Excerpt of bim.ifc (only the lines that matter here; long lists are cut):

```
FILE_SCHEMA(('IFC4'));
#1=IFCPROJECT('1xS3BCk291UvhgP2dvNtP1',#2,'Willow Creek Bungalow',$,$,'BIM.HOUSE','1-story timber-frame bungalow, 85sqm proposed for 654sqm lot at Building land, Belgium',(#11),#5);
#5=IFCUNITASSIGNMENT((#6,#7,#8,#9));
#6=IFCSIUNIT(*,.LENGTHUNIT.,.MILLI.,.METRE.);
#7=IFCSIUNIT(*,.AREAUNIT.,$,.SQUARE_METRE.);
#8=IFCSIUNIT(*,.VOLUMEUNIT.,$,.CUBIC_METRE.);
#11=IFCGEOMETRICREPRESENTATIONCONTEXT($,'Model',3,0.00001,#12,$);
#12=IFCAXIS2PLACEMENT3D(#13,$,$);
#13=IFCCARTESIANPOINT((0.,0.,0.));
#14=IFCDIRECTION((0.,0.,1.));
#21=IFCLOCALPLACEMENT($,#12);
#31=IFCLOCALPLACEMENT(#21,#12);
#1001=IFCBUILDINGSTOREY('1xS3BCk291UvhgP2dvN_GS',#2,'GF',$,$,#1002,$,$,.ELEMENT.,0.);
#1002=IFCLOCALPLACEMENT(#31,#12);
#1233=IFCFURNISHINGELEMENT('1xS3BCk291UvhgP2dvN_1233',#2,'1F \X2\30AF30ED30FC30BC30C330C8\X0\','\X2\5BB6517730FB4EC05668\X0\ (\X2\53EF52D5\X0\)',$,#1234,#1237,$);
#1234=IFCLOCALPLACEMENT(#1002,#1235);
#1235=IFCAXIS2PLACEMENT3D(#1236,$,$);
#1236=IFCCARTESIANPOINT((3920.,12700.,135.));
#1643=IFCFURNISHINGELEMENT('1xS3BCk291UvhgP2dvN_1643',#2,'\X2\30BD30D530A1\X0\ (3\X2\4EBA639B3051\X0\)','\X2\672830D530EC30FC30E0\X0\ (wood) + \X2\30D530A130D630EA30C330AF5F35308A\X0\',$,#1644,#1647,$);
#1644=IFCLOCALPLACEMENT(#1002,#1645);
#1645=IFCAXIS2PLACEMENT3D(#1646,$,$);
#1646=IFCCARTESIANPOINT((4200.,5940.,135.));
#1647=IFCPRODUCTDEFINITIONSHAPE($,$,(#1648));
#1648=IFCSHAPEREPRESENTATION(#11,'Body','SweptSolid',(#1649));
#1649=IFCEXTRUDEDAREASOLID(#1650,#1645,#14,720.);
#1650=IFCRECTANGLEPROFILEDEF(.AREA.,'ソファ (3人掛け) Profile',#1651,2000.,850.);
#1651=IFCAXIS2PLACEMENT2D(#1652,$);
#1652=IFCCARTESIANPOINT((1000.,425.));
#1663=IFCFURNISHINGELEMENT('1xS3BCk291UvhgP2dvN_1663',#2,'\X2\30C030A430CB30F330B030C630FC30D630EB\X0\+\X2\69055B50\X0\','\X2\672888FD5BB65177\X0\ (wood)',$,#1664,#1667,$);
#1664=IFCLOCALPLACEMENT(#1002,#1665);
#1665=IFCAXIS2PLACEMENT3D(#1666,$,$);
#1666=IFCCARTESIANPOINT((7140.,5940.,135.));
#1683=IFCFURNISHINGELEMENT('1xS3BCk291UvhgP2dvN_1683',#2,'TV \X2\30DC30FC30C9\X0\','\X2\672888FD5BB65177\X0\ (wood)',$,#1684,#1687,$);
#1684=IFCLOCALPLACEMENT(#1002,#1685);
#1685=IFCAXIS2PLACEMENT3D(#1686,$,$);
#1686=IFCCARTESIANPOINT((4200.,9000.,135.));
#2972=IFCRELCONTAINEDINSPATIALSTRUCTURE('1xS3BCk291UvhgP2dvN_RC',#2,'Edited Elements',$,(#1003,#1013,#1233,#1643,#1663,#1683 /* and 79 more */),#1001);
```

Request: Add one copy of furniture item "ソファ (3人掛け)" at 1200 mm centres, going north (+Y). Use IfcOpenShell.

```python
import numpy as np
import ifcopenshell
import ifcopenshell.api.geometry
import ifcopenshell.api.root
import ifcopenshell.util.element
import ifcopenshell.util.placement
import ifcopenshell.util.unit

model = ifcopenshell.open("bim.ifc")
unit_scale = ifcopenshell.util.unit.calculate_unit_scale(model)


def reuse_history(source, copy):
    """copy_class also copies each property set's owner history, people and application; keep the originals."""
    for rel in copy.IsDefinedBy:
        if rel.is_a("IfcRelDefinesByProperties") and (history := rel.RelatingPropertyDefinition.OwnerHistory):
            rel.RelatingPropertyDefinition.OwnerHistory = source.OwnerHistory
            ifcopenshell.util.element.remove_deep2(model, history)


source = model.by_guid("1xS3BCk291UvhgP2dvN_1643")
base = ifcopenshell.util.placement.get_local_placement(source.ObjectPlacement)
step = np.array([0.0, 1.0, 0.0]) * 1.2 / unit_scale

for i in range(1, 2):
    copy = ifcopenshell.api.root.copy_class(model, product=source)
    copy.Representation = ifcopenshell.util.element.copy_deep(
        model, source.Representation, exclude=["IfcGeometricRepresentationContext", "IfcRepresentationMap"]
    )
    reuse_history(source, copy)
    matrix = base.copy()
    matrix[:3, 3] += i * step
    print("added at", matrix[:3, 3].round(3) + 0.0)
    ifcopenshell.api.geometry.edit_object_placement(model, product=copy, matrix=matrix, is_si=False)

model.write("bim_updated.ifc")
```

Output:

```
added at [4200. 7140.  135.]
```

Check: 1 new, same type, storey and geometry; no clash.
